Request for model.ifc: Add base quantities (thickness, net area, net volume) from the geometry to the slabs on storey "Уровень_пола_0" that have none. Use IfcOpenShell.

First a look at what the model holds.

```python
import ifcopenshell
import ifcopenshell.util.element
import ifcopenshell.util.unit

model = ifcopenshell.open("model.ifc")
print(model.schema)
for unit_type in ("LENGTHUNIT", "AREAUNIT", "VOLUMEUNIT"):
    print(unit_type, ifcopenshell.util.unit.calculate_unit_scale(model, unit_type))
storey = next(s for s in model.by_type("IfcBuildingStorey") if s.Name == "Уровень_пола_0")
slabs = [e for e in ifcopenshell.util.element.get_decomposition(storey) if e.is_a("IfcSlab")]
for e in sorted(slabs, key=lambda e: e.id()):
    print(e.id(), e.is_a(), e.Name, list(ifcopenshell.util.element.get_psets(e, qtos_only=True)), sep=" | ")
```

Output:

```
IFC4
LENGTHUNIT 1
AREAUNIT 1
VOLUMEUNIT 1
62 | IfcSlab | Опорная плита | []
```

```python
import ifcopenshell
import ifcopenshell.api.pset
import ifcopenshell.geom
import ifcopenshell.util.element
import ifcopenshell.util.shape
import ifcopenshell.util.unit

model = ifcopenshell.open("model.ifc")
unit_scale = ifcopenshell.util.unit.calculate_unit_scale(model)
area_scale = ifcopenshell.util.unit.calculate_unit_scale(model, "AREAUNIT")
volume_scale = ifcopenshell.util.unit.calculate_unit_scale(model, "VOLUMEUNIT")
settings = ifcopenshell.geom.settings()

storey = next(s for s in model.by_type("IfcBuildingStorey") if s.Name == "Уровень_пола_0")
slabs = [e for e in ifcopenshell.util.element.get_decomposition(storey) if e.is_a("IfcSlab")]

for e in sorted(slabs, key=lambda e: e.id()):
    if ifcopenshell.util.element.get_psets(e, qtos_only=True, should_inherit=False):
        continue
    # Geometry comes back in metres, in the element's own axes.
    shape = ifcopenshell.geom.create_shape(settings, e)
    values = {
        "Width": ifcopenshell.util.shape.get_z(shape.geometry) / unit_scale,
        "NetArea": ifcopenshell.util.shape.get_footprint_area(shape.geometry) / area_scale,
        "NetVolume": ifcopenshell.util.shape.get_volume(shape.geometry) / volume_scale,
    }
    qto = ifcopenshell.api.pset.add_qto(model, product=e, name="Qto_SlabBaseQuantities")
    ifcopenshell.api.pset.edit_qto(model, qto=qto, properties=values)
    print(e.id(), {k: round(v, 3) for k, v in values.items()})

model.write("model_updated.ifc")
```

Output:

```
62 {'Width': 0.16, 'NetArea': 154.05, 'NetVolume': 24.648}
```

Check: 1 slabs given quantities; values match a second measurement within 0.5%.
